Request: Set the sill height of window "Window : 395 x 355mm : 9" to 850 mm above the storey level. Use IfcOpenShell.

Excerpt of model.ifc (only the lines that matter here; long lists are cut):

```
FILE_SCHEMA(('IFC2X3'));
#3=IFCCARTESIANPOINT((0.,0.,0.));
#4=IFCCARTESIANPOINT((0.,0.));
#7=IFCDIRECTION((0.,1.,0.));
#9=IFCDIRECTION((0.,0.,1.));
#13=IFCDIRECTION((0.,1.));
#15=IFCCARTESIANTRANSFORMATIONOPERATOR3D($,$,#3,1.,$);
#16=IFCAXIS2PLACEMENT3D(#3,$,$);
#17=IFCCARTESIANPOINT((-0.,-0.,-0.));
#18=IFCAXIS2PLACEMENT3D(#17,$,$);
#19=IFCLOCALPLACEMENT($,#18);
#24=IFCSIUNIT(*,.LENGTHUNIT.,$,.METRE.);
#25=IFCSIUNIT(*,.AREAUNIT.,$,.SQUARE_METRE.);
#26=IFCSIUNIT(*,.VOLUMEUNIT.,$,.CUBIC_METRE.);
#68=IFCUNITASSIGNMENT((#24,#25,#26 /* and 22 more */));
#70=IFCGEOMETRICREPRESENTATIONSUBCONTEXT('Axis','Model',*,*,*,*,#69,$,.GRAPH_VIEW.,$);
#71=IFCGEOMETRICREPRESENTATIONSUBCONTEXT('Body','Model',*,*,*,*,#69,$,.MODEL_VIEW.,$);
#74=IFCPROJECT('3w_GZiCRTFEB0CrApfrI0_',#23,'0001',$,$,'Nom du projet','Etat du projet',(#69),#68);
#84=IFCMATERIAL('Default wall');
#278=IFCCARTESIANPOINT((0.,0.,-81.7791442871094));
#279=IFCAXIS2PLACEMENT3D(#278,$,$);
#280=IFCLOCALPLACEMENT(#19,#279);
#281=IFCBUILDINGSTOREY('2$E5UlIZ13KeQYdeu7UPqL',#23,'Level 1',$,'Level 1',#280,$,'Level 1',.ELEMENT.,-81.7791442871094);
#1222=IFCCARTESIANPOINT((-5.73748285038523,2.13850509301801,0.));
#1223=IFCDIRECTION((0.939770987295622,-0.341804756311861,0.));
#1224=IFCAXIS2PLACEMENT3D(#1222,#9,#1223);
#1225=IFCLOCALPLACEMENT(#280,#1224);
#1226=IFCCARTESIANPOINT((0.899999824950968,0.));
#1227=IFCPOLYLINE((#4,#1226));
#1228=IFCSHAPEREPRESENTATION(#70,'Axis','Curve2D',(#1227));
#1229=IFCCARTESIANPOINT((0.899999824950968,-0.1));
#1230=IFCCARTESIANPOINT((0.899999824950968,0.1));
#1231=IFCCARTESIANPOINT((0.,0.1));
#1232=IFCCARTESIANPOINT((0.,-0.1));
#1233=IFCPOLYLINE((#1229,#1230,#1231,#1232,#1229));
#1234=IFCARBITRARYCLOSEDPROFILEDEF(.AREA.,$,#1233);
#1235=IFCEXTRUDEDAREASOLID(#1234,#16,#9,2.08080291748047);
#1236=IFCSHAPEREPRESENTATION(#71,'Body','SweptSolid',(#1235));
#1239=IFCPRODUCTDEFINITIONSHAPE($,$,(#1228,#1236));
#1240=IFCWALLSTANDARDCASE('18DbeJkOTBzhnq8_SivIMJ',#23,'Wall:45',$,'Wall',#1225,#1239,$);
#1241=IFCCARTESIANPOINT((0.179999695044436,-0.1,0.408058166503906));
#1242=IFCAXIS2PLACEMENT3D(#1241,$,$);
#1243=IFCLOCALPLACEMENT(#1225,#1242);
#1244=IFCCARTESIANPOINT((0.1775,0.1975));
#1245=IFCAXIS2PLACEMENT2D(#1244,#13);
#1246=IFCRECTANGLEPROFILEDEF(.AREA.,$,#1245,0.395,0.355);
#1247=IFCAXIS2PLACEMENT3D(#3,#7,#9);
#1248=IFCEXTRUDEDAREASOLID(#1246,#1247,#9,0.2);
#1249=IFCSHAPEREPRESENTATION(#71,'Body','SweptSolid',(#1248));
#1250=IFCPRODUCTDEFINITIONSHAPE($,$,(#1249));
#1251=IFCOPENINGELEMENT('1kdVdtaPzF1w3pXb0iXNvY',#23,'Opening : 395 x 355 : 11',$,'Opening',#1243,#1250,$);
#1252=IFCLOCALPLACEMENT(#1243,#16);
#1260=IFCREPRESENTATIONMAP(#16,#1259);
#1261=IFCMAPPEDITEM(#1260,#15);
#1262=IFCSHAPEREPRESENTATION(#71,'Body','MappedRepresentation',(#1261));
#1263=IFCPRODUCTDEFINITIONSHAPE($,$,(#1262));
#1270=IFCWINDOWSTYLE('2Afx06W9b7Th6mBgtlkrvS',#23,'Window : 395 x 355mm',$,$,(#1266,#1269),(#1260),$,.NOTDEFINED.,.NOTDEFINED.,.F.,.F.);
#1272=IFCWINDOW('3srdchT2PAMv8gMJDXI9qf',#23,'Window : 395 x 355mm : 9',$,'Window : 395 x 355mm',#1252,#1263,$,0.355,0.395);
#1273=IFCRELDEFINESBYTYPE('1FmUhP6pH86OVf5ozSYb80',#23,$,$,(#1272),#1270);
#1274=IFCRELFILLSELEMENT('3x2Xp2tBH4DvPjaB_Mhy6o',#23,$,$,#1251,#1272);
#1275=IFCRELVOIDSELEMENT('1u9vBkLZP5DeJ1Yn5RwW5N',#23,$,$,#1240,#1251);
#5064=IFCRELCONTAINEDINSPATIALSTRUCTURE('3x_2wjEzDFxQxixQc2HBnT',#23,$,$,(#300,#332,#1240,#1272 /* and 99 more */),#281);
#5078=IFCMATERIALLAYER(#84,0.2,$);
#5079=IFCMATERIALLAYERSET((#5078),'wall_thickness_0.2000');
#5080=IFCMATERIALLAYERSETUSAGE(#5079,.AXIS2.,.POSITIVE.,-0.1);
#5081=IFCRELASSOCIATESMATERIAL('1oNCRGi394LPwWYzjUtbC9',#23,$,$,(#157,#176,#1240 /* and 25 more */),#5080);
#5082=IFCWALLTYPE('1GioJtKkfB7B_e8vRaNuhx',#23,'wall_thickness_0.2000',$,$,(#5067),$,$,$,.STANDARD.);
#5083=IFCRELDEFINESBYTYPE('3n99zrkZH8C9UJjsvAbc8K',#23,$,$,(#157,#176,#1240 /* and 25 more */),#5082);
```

```python
import numpy as np
import ifcopenshell
import ifcopenshell.api.geometry
import ifcopenshell.geom
import ifcopenshell.util.element
import ifcopenshell.util.placement
import ifcopenshell.util.shape
import ifcopenshell.util.unit

model = ifcopenshell.open("model.ifc")
unit_scale = ifcopenshell.util.unit.calculate_unit_scale(model)

window = model.by_guid("3srdchT2PAMv8gMJDXI9qf")
opening = window.FillsVoids[0].RelatingOpeningElement
storey = ifcopenshell.util.element.get_container(window, ifc_class="IfcBuildingStorey")
level = ifcopenshell.util.placement.get_local_placement(storey.ObjectPlacement)[2, 3]

# The opening's origin need not be at the sill, so measure its lowest point.
shape = ifcopenshell.geom.create_shape(ifcopenshell.geom.settings(), opening)
bottom = ifcopenshell.util.shape.get_shape_bottom_elevation(shape, shape.geometry) / unit_scale
dz = level + 0.85 / unit_scale - bottom

shift = np.array([0.0, 0.0, dz])
# The window is placed relative to its opening, so it follows when the opening moves.
matrix = ifcopenshell.util.placement.get_local_placement(opening.ObjectPlacement)
matrix[:3, 3] += shift
ifcopenshell.api.geometry.edit_object_placement(
    model, product=opening, matrix=matrix, is_si=False, should_transform_children=True
)

print(f"moved by {dz * unit_scale:+.3f} m")

model.write("model_edited.ifc")
```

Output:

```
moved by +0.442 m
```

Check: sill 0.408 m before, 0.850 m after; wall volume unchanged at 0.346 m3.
